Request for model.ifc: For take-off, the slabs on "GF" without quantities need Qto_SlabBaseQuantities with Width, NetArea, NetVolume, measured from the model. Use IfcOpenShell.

First a look at what the model holds.

```python
import ifcopenshell
import ifcopenshell.util.element
import ifcopenshell.util.unit

model = ifcopenshell.open("model.ifc")
print(model.schema)
for unit_type in ("LENGTHUNIT", "AREAUNIT", "VOLUMEUNIT"):
    print(unit_type, ifcopenshell.util.unit.calculate_unit_scale(model, unit_type))
storey = next(s for s in model.by_type("IfcBuildingStorey") if s.Name == "GF")
slabs = [e for e in ifcopenshell.util.element.get_decomposition(storey) if e.is_a("IfcSlab")]
for e in sorted(slabs, key=lambda e: e.id()):
    print(e.id(), e.is_a(), e.Name, list(ifcopenshell.util.element.get_psets(e, qtos_only=True)), sep=" | ")
```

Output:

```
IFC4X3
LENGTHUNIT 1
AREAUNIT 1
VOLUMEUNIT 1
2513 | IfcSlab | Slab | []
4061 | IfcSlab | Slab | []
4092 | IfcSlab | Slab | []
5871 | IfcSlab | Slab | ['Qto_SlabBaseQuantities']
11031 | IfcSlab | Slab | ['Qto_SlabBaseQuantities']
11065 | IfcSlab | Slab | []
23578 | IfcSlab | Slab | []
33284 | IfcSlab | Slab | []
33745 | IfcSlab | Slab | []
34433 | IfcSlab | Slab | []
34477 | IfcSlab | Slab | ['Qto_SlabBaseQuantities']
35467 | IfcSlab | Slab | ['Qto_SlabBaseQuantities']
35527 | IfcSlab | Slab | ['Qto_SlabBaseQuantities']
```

```python
import ifcopenshell
import ifcopenshell.api.pset
import ifcopenshell.geom
import ifcopenshell.util.element
import ifcopenshell.util.shape
import ifcopenshell.util.unit

model = ifcopenshell.open("model.ifc")
unit_scale = ifcopenshell.util.unit.calculate_unit_scale(model)
area_scale = ifcopenshell.util.unit.calculate_unit_scale(model, "AREAUNIT")
volume_scale = ifcopenshell.util.unit.calculate_unit_scale(model, "VOLUMEUNIT")
settings = ifcopenshell.geom.settings()

storey = next(s for s in model.by_type("IfcBuildingStorey") if s.Name == "GF")
slabs = [e for e in ifcopenshell.util.element.get_decomposition(storey) if e.is_a("IfcSlab")]

for e in sorted(slabs, key=lambda e: e.id()):
    if ifcopenshell.util.element.get_psets(e, qtos_only=True, should_inherit=False):
        continue
    # Geometry comes back in metres, in the element's own axes.
    shape = ifcopenshell.geom.create_shape(settings, e)
    values = {
        "Width": ifcopenshell.util.shape.get_z(shape.geometry) / unit_scale,
        "NetArea": ifcopenshell.util.shape.get_footprint_area(shape.geometry) / area_scale,
        "NetVolume": ifcopenshell.util.shape.get_volume(shape.geometry) / volume_scale,
    }
    qto = ifcopenshell.api.pset.add_qto(model, product=e, name="Qto_SlabBaseQuantities")
    ifcopenshell.api.pset.edit_qto(model, qto=qto, properties=values)
    print(e.id(), {k: round(v, 3) for k, v in values.items()})

model.write("model_rev.ifc")
```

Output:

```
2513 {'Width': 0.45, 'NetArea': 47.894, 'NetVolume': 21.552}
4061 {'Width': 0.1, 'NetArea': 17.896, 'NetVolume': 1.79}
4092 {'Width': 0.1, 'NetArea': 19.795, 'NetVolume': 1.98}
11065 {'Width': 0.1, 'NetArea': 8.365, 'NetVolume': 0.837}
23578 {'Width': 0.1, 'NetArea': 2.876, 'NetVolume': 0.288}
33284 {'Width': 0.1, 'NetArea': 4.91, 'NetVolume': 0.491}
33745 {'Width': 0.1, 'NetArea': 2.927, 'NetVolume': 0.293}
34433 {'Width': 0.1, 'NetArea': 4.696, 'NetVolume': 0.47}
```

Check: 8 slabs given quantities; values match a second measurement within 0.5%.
